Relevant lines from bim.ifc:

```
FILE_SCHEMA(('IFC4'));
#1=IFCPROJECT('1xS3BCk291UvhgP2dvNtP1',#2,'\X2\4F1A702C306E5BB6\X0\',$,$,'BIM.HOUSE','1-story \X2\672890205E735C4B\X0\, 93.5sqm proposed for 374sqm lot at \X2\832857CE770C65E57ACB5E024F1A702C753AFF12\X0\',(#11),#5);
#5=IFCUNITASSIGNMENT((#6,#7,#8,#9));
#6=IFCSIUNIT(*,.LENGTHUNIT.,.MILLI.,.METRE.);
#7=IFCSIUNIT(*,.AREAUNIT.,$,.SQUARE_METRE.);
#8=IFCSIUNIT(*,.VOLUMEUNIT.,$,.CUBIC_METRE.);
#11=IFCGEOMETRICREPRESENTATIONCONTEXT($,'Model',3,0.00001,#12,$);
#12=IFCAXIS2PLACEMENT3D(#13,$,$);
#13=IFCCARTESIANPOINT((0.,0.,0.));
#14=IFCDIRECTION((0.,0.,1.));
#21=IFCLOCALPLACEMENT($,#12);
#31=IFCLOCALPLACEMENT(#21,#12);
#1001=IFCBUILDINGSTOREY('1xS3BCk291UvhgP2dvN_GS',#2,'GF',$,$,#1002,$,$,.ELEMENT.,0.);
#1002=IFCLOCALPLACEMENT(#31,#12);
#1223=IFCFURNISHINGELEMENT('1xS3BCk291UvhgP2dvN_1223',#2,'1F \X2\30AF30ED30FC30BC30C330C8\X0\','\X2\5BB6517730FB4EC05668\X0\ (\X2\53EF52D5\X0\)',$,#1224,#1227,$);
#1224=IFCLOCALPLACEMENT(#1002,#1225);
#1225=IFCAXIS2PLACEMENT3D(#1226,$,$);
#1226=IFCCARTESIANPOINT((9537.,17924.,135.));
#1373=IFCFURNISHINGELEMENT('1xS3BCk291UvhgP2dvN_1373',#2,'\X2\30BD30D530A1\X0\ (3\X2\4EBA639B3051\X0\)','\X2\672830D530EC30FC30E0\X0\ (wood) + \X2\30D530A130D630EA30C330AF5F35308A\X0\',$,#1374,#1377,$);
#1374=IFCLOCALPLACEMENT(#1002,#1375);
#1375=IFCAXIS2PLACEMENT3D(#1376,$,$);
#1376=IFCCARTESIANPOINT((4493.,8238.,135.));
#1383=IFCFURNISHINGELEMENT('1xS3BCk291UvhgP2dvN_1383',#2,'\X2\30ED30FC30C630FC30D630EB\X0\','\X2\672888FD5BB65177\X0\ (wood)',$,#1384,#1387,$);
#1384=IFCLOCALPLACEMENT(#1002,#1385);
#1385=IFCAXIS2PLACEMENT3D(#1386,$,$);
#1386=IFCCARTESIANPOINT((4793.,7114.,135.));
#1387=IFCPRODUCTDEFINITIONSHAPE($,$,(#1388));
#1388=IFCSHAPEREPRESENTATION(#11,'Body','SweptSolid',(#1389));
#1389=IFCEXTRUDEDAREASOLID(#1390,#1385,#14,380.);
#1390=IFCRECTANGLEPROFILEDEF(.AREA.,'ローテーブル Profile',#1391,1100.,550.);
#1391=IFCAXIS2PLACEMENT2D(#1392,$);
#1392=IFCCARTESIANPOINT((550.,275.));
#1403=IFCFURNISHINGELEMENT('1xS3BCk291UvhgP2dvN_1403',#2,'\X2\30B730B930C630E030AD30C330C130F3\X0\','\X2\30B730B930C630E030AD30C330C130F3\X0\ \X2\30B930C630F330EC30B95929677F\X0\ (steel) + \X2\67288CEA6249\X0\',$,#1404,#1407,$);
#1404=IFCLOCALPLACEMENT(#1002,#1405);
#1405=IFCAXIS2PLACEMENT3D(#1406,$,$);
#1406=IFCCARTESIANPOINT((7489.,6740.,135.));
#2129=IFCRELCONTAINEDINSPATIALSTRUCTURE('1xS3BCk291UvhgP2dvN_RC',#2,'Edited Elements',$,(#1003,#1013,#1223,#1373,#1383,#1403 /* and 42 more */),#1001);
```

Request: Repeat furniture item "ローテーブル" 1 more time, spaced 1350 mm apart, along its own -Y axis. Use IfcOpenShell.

```python
import ifcopenshell
import ifcopenshell.api.geometry
import ifcopenshell.api.root
import ifcopenshell.util.element
import ifcopenshell.util.placement
import ifcopenshell.util.unit

model = ifcopenshell.open("bim.ifc")
unit_scale = ifcopenshell.util.unit.calculate_unit_scale(model)


def reuse_history(source, copy):
    """copy_class also copies each property set's owner history, people and application; keep the originals."""
    for rel in copy.IsDefinedBy:
        if rel.is_a("IfcRelDefinesByProperties") and (history := rel.RelatingPropertyDefinition.OwnerHistory):
            rel.RelatingPropertyDefinition.OwnerHistory = source.OwnerHistory
            ifcopenshell.util.element.remove_deep2(model, history)


source = model.by_guid("1xS3BCk291UvhgP2dvN_1383")
base = ifcopenshell.util.placement.get_local_placement(source.ObjectPlacement)
step = -base[:3, 1] * 1.35 / unit_scale

for i in range(1, 2):
    copy = ifcopenshell.api.root.copy_class(model, product=source)
    copy.Representation = ifcopenshell.util.element.copy_deep(
        model, source.Representation, exclude=["IfcGeometricRepresentationContext", "IfcRepresentationMap"]
    )
    reuse_history(source, copy)
    matrix = base.copy()
    matrix[:3, 3] += i * step
    print("added at", matrix[:3, 3].round(3) + 0.0)
    ifcopenshell.api.geometry.edit_object_placement(model, product=copy, matrix=matrix, is_si=False)

model.write("bim-out.ifc")
```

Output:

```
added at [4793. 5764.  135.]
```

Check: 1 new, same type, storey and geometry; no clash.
